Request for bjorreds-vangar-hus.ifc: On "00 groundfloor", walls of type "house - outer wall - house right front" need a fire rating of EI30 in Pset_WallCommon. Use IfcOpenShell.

First a look at what the model holds.

```python
import ifcopenshell
import ifcopenshell.util.element

model = ifcopenshell.open("bjorreds-vangar-hus.ifc")
print(model.schema)
storey = next(s for s in model.by_type("IfcBuildingStorey") if s.Name == "00 groundfloor")
walls = [e for e in ifcopenshell.util.element.get_decomposition(storey) if e.is_a("IfcWall")]
seen = {}
for e in walls:
    element_type = ifcopenshell.util.element.get_type(e)
    key = (element_type.Name if element_type != e and element_type else None, ifcopenshell.util.element.get_pset(e, "Pset_WallCommon", "FireRating"))
    seen[key] = seen.get(key, 0) + 1
for (name, value), count in sorted(seen.items(), key=str):
    print(count, "x", name, "|", value)
```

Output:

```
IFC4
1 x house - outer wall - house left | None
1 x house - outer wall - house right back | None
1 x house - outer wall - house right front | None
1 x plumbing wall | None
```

```python
import ifcopenshell
import ifcopenshell.api.pset
import ifcopenshell.util.element

model = ifcopenshell.open("bjorreds-vangar-hus.ifc")

storey = next(s for s in model.by_type("IfcBuildingStorey") if s.Name == "00 groundfloor")
walls = [e for e in ifcopenshell.util.element.get_decomposition(storey) if e.is_a("IfcWall")]

count = 0
for e in walls:
    element_type = ifcopenshell.util.element.get_type(e)
    if element_type in (None, e) or element_type.Name != "house - outer wall - house right front":
        continue
    # add_pset returns the element's existing set when there is one.
    pset = ifcopenshell.api.pset.add_pset(model, product=e, name="Pset_WallCommon")
    ifcopenshell.api.pset.edit_pset(model, pset=pset, properties={"FireRating": "EI30"})
    count += 1

print(count, "walls updated")

model.write("bjorreds-vangar-hus_edited.ifc")
```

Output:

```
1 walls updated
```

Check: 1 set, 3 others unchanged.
